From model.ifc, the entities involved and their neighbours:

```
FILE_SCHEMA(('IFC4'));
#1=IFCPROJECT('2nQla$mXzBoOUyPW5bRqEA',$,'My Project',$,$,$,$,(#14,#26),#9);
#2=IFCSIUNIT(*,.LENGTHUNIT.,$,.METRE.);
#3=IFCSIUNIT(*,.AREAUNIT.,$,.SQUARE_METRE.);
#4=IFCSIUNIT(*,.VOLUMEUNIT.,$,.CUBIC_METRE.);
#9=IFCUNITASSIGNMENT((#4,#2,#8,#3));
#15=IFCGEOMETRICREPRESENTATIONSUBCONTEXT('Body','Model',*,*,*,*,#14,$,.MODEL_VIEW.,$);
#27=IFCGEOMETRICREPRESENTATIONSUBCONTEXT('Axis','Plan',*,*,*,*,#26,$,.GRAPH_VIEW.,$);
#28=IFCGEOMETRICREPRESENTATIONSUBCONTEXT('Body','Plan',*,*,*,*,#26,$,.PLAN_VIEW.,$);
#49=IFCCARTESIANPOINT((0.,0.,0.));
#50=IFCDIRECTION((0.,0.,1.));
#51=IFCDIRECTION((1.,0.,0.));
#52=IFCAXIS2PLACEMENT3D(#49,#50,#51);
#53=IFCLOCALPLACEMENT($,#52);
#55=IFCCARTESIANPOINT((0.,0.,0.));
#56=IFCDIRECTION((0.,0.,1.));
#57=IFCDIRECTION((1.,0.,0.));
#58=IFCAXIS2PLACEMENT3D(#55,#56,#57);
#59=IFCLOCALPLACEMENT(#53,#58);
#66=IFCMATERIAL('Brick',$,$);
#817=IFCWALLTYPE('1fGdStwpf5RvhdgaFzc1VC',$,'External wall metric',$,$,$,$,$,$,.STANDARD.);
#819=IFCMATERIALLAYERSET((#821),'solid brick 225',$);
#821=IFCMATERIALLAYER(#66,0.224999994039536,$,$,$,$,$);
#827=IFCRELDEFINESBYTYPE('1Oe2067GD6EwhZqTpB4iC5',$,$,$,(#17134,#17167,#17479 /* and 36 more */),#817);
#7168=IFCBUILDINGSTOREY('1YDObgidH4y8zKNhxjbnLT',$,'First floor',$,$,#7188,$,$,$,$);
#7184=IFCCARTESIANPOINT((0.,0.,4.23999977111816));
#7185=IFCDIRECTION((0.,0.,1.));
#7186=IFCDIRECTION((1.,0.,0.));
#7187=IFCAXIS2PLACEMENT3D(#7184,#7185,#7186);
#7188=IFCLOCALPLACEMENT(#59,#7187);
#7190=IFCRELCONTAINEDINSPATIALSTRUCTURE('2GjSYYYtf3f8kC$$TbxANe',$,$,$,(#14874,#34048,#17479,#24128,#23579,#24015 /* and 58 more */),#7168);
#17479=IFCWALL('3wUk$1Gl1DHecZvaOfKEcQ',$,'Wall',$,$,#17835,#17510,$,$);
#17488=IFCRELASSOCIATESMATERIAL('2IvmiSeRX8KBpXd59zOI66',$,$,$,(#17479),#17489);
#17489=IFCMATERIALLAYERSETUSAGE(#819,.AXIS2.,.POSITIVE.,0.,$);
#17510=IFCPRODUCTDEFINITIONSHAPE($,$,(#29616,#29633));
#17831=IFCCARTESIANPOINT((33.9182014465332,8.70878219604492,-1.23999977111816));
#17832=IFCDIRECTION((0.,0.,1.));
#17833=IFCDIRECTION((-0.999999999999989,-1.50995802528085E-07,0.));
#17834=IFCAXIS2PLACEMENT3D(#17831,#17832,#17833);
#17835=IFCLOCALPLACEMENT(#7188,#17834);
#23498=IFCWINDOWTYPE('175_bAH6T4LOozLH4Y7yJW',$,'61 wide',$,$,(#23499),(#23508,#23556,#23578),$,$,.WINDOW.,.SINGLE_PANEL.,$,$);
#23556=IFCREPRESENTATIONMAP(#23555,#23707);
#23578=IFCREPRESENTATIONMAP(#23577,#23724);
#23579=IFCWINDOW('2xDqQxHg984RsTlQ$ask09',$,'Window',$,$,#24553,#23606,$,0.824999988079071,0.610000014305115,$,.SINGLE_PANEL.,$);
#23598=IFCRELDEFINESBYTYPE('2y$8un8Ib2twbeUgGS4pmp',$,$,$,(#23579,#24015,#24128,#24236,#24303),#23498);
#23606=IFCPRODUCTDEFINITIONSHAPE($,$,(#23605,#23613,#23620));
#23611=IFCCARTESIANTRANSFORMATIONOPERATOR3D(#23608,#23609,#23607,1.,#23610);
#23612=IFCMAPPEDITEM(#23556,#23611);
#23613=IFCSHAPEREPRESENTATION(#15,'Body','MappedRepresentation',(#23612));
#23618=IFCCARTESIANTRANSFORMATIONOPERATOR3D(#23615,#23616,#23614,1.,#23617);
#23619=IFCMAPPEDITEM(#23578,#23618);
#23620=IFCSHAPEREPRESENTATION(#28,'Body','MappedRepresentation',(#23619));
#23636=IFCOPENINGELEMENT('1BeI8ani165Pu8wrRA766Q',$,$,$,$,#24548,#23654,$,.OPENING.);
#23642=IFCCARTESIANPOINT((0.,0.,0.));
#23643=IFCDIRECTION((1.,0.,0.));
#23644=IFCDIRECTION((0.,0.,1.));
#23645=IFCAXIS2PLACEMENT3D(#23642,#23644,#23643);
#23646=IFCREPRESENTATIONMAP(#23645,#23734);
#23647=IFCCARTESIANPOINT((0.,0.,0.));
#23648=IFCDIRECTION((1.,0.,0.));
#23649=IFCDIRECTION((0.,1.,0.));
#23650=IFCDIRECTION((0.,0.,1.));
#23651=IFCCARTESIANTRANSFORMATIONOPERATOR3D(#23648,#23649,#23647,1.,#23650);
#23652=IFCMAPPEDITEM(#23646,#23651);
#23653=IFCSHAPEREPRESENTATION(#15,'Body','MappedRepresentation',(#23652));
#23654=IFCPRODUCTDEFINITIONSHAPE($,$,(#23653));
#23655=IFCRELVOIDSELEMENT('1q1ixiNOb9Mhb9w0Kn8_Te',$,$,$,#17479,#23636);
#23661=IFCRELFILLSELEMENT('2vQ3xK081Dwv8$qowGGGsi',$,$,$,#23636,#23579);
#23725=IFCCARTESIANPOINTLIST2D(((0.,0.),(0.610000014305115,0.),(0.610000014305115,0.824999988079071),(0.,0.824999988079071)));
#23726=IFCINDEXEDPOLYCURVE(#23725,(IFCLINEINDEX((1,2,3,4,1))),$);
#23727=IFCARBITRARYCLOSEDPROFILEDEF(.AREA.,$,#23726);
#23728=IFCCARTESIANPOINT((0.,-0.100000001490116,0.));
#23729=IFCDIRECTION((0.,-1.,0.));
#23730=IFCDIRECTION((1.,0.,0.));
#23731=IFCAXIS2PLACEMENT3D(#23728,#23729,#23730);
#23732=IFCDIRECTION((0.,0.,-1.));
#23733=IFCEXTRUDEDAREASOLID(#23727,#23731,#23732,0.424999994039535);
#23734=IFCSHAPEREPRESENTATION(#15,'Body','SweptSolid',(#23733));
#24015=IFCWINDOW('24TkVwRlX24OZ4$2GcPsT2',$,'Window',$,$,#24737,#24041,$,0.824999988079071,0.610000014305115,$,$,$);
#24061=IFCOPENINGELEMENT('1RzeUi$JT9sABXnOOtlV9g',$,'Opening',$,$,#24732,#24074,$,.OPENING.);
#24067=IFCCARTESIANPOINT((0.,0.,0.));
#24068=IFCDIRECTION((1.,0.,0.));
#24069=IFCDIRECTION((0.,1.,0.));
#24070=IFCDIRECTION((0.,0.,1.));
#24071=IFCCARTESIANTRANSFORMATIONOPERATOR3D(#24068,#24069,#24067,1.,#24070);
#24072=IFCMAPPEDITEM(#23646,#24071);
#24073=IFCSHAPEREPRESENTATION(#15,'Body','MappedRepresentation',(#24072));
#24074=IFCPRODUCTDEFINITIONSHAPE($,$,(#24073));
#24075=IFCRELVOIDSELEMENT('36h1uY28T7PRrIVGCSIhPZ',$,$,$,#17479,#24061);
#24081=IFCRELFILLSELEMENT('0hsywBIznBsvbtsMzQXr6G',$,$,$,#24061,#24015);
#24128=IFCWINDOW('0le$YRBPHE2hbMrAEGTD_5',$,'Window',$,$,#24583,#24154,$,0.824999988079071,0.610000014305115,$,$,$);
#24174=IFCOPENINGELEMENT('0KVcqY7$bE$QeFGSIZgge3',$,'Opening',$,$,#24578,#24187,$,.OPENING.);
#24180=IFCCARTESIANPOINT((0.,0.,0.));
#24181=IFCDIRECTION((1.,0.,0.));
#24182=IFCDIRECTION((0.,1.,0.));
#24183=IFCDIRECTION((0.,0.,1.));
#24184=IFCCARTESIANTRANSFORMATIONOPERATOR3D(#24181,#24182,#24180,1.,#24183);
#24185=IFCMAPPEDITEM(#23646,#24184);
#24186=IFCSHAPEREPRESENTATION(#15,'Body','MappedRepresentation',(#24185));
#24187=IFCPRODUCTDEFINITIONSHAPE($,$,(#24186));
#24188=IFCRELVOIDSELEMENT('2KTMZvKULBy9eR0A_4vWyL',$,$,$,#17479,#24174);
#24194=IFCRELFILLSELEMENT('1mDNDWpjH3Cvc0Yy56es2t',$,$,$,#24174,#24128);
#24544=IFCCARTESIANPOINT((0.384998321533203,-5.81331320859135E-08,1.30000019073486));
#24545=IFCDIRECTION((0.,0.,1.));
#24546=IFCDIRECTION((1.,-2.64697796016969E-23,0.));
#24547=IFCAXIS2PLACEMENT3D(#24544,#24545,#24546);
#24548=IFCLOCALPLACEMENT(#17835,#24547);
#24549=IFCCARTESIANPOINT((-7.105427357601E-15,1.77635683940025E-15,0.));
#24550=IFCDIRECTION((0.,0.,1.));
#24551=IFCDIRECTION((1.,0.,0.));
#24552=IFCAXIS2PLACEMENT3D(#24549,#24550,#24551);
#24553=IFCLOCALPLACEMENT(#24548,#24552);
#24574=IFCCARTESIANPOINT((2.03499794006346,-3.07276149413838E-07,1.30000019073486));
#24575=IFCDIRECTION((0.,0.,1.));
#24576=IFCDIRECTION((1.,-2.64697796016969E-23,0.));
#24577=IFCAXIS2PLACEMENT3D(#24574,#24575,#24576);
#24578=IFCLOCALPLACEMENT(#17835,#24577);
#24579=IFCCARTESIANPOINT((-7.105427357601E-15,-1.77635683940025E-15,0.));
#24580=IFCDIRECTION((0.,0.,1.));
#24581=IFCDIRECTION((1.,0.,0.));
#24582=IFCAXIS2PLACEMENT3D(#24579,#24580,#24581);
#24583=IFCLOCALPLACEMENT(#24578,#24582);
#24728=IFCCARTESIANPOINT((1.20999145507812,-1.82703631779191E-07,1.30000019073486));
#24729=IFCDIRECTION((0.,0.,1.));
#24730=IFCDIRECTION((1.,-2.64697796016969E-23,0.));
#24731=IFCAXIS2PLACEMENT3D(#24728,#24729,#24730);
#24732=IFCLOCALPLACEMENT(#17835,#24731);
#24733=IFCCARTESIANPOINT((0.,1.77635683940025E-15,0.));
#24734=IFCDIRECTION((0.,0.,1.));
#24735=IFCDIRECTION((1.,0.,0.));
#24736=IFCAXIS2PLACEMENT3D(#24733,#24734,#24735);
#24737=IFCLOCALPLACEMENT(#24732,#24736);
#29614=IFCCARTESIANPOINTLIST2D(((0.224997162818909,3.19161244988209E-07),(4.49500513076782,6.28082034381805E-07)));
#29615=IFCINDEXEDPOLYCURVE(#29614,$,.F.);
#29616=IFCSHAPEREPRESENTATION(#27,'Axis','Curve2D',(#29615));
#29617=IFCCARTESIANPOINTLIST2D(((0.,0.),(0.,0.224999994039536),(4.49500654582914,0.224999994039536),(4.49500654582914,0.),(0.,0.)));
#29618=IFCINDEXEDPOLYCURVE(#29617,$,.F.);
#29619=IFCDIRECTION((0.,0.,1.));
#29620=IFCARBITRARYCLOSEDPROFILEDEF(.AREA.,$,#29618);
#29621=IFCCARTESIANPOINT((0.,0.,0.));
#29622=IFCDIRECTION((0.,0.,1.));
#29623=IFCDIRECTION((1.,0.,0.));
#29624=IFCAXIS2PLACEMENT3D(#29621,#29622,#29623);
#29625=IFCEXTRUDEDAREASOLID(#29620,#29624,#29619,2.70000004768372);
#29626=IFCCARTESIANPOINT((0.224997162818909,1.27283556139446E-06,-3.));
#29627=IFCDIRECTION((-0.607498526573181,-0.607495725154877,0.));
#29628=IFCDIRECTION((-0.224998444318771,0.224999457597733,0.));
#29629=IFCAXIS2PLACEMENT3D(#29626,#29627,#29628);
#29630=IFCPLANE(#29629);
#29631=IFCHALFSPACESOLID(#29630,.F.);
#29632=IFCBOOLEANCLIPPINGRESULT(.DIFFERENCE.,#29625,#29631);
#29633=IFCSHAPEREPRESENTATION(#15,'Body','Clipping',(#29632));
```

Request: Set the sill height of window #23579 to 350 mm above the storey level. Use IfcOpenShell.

```python
import numpy as np
import ifcopenshell
import ifcopenshell.api.geometry
import ifcopenshell.geom
import ifcopenshell.util.element
import ifcopenshell.util.placement
import ifcopenshell.util.shape
import ifcopenshell.util.unit

model = ifcopenshell.open("model.ifc")
unit_scale = ifcopenshell.util.unit.calculate_unit_scale(model)

window = model.by_id(23579)
opening = window.FillsVoids[0].RelatingOpeningElement
storey = ifcopenshell.util.element.get_container(window, ifc_class="IfcBuildingStorey")
level = ifcopenshell.util.placement.get_local_placement(storey.ObjectPlacement)[2, 3]

# The opening's origin need not be at the sill, so measure its lowest point.
shape = ifcopenshell.geom.create_shape(ifcopenshell.geom.settings(), opening)
bottom = ifcopenshell.util.shape.get_shape_bottom_elevation(shape, shape.geometry) / unit_scale
dz = level + 0.35 - bottom

shift = np.array([0.0, 0.0, dz])
# The window is placed relative to its opening, so it follows when the opening moves.
matrix = ifcopenshell.util.placement.get_local_placement(opening.ObjectPlacement)
matrix[:3, 3] += shift
ifcopenshell.api.geometry.edit_object_placement(
    model, product=opening, matrix=matrix, is_si=False, should_transform_children=True
)

print(f"moved by {dz * unit_scale:+.3f} m")

model.write("model_updated.ifc")
```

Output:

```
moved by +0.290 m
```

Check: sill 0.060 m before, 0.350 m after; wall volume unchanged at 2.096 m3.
